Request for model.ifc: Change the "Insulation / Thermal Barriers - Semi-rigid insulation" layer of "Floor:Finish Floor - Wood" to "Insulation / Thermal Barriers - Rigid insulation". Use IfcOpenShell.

First a look at what the model holds.

```python
import ifcopenshell
import ifcopenshell.util.element

model = ifcopenshell.open("model.ifc")
print(model.schema)
for layer_set in model.by_type("IfcMaterialLayerSet"):
    if layer_set.LayerSetName == "Floor:Finish Floor - Wood":
        for layer in layer_set.MaterialLayers:
            print(layer.id(), layer.Material and layer.Material.Name, layer.LayerThickness, sep=" | ")
        print(len(ifcopenshell.util.element.get_elements_by_material(model, layer_set)), "elements and types use it")
print(sorted(m.Name for m in model.by_type("IfcMaterial") if m.Name)[:60])
```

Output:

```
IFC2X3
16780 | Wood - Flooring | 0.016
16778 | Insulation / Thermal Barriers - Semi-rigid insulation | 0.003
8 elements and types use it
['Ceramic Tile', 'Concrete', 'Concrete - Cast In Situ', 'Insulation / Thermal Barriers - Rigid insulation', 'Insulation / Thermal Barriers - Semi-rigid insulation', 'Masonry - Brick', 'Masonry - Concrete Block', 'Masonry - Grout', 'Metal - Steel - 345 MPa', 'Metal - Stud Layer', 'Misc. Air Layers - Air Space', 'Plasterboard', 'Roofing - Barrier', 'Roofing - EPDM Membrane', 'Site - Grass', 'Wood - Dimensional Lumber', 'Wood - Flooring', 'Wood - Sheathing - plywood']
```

```python
import ifcopenshell
import ifcopenshell.api.material

model = ifcopenshell.open("model.ifc")

layer_set = next(s for s in model.by_type("IfcMaterialLayerSet") if s.LayerSetName == "Floor:Finish Floor - Wood")
layer = next(l for l in layer_set.MaterialLayers if l.Material and l.Material.Name == "Insulation / Thermal Barriers - Semi-rigid insulation")
material = next(m for m in model.by_type("IfcMaterial") if m.Name == "Insulation / Thermal Barriers - Rigid insulation")

# Point this one layer at the other material; renaming the old one would change it everywhere.
ifcopenshell.api.material.edit_layer(model, layer=layer, attributes={}, material=material)

print([l.Material.Name if l.Material else None for l in layer_set.MaterialLayers])

model.write("model_edited.ifc")
```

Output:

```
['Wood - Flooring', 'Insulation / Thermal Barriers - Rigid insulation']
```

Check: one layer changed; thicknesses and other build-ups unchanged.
